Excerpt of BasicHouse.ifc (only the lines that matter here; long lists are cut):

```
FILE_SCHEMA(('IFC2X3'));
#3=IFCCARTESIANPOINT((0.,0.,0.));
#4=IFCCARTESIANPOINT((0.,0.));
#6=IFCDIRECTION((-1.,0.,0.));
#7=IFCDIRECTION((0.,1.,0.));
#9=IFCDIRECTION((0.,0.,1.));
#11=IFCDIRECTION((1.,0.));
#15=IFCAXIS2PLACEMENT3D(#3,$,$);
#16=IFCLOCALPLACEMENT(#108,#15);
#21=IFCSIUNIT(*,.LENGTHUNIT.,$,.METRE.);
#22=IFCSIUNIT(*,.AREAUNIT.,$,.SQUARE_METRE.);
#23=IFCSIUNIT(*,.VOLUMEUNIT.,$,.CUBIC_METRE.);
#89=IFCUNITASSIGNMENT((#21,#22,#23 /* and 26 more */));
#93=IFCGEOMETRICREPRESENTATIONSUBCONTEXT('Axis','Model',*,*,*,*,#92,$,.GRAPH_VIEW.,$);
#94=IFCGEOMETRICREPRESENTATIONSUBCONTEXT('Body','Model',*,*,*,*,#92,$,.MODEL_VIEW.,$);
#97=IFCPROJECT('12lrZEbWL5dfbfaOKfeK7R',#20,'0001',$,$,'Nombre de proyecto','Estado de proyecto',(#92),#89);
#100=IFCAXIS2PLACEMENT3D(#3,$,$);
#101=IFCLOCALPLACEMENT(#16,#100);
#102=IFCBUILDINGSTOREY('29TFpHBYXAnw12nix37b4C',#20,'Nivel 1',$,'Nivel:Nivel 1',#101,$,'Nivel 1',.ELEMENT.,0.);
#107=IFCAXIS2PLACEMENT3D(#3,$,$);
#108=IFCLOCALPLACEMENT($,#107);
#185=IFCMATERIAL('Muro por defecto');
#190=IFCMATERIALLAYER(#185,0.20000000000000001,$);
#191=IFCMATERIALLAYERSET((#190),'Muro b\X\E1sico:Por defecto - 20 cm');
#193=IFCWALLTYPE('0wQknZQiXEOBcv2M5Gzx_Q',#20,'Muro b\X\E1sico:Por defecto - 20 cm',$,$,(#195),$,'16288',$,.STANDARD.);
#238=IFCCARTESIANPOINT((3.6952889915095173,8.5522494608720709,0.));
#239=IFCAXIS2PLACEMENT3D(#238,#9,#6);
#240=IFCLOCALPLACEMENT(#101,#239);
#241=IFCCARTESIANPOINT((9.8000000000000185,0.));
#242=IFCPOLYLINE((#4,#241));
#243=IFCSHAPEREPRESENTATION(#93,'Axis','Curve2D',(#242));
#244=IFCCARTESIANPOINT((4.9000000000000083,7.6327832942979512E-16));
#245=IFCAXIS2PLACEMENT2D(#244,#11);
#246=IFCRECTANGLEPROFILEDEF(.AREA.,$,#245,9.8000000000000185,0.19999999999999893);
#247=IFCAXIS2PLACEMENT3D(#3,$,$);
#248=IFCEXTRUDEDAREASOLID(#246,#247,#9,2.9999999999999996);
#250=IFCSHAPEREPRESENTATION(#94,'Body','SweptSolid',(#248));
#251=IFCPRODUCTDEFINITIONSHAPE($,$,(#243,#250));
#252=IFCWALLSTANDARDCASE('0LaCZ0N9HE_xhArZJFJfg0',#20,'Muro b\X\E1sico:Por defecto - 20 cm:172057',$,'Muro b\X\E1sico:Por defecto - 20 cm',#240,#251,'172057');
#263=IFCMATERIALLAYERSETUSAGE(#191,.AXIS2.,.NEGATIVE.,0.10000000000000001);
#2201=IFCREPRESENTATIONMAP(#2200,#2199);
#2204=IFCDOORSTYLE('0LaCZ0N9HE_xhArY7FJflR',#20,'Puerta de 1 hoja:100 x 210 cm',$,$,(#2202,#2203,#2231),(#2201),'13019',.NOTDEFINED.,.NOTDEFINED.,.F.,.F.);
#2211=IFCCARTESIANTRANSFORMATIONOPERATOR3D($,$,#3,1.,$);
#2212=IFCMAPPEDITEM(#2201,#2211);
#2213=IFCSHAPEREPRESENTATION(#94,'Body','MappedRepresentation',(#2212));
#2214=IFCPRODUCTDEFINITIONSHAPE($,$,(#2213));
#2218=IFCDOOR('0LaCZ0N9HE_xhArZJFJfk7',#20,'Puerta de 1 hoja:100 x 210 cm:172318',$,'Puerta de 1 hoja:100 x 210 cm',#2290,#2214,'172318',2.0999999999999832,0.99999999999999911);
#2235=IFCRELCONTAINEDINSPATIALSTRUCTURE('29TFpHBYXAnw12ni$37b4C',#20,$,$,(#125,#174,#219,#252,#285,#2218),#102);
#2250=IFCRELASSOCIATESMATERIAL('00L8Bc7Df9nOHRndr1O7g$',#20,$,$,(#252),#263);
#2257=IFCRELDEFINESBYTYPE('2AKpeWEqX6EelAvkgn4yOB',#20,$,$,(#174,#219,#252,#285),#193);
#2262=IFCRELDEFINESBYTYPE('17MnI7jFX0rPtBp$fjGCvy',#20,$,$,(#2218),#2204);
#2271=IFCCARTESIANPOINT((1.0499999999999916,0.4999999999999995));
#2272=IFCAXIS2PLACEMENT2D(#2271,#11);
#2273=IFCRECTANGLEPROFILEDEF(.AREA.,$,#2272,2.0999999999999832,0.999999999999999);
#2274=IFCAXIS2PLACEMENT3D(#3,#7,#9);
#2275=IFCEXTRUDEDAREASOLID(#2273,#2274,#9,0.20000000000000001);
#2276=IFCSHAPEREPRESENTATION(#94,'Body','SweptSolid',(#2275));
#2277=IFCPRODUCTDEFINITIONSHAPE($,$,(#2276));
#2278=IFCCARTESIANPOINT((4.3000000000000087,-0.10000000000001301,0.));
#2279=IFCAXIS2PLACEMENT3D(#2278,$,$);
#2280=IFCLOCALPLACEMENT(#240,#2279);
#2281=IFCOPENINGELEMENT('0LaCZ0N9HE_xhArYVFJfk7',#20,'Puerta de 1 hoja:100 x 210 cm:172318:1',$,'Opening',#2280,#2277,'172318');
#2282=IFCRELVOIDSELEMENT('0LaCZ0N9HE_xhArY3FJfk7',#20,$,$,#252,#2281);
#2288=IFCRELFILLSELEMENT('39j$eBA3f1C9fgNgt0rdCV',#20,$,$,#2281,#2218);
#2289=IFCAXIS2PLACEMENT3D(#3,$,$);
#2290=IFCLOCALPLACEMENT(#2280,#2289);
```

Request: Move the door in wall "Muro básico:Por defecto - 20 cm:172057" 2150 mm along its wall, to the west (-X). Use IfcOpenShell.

```python
import ifcopenshell
import ifcopenshell.api.geometry
import ifcopenshell.util.placement

model = ifcopenshell.open("BasicHouse.ifc")

door = model.by_guid("0LaCZ0N9HE_xhArZJFJfk7")
opening = door.FillsVoids[0].RelatingOpeningElement
wall = opening.VoidsElements[0].RelatingBuildingElement

wall_matrix = ifcopenshell.util.placement.get_local_placement(wall.ObjectPlacement)
shift = wall_matrix[:3, 0] * 2.15
before = ifcopenshell.util.placement.get_local_placement(door.ObjectPlacement)[:3, 3].copy()

# The door is placed relative to its opening, so it follows when the opening moves.
matrix = ifcopenshell.util.placement.get_local_placement(opening.ObjectPlacement)
matrix[:3, 3] += shift
ifcopenshell.api.geometry.edit_object_placement(
    model, product=opening, matrix=matrix, is_si=False, should_transform_children=True
)

after = ifcopenshell.util.placement.get_local_placement(door.ObjectPlacement)[:3, 3]
print("door moved by", (after - before).round(3) + 0.0)

model.write("BasicHouse_edited.ifc")
```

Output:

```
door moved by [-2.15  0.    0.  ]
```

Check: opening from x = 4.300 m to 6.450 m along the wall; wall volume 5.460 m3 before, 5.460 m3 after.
